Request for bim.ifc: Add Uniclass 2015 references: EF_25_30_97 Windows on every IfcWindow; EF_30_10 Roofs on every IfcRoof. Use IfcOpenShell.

First a look at what the model holds.

```python
import ifcopenshell

model = ifcopenshell.open("bim.ifc")
print(model.schema)
print("classifications:", [c.Name for c in model.by_type("IfcClassification")])
for ifc_class in ("IfcDoor", "IfcRoof", "IfcStair", "IfcWall", "IfcWindow"):
    print(ifc_class, len(model.by_type(ifc_class)))
```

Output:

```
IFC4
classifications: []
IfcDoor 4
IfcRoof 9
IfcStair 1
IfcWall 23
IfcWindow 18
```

```python
import ifcopenshell
import ifcopenshell.api.classification

model = ifcopenshell.open("bim.ifc")

system = ifcopenshell.api.classification.add_classification(model, classification="Uniclass 2015")

codes = {
    "IfcWindow": ("EF_25_30_97", "Windows"),
    "IfcRoof": ("EF_30_10", "Roofs"),
}
for ifc_class, (code, name) in codes.items():
    products = model.by_type(ifc_class)
    ifcopenshell.api.classification.add_reference(
        model, products=products, classification=system, identification=code, name=name
    )
    print(code, len(products))

model.write("bim_edited.ifc")
```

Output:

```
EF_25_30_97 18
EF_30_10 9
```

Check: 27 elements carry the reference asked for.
